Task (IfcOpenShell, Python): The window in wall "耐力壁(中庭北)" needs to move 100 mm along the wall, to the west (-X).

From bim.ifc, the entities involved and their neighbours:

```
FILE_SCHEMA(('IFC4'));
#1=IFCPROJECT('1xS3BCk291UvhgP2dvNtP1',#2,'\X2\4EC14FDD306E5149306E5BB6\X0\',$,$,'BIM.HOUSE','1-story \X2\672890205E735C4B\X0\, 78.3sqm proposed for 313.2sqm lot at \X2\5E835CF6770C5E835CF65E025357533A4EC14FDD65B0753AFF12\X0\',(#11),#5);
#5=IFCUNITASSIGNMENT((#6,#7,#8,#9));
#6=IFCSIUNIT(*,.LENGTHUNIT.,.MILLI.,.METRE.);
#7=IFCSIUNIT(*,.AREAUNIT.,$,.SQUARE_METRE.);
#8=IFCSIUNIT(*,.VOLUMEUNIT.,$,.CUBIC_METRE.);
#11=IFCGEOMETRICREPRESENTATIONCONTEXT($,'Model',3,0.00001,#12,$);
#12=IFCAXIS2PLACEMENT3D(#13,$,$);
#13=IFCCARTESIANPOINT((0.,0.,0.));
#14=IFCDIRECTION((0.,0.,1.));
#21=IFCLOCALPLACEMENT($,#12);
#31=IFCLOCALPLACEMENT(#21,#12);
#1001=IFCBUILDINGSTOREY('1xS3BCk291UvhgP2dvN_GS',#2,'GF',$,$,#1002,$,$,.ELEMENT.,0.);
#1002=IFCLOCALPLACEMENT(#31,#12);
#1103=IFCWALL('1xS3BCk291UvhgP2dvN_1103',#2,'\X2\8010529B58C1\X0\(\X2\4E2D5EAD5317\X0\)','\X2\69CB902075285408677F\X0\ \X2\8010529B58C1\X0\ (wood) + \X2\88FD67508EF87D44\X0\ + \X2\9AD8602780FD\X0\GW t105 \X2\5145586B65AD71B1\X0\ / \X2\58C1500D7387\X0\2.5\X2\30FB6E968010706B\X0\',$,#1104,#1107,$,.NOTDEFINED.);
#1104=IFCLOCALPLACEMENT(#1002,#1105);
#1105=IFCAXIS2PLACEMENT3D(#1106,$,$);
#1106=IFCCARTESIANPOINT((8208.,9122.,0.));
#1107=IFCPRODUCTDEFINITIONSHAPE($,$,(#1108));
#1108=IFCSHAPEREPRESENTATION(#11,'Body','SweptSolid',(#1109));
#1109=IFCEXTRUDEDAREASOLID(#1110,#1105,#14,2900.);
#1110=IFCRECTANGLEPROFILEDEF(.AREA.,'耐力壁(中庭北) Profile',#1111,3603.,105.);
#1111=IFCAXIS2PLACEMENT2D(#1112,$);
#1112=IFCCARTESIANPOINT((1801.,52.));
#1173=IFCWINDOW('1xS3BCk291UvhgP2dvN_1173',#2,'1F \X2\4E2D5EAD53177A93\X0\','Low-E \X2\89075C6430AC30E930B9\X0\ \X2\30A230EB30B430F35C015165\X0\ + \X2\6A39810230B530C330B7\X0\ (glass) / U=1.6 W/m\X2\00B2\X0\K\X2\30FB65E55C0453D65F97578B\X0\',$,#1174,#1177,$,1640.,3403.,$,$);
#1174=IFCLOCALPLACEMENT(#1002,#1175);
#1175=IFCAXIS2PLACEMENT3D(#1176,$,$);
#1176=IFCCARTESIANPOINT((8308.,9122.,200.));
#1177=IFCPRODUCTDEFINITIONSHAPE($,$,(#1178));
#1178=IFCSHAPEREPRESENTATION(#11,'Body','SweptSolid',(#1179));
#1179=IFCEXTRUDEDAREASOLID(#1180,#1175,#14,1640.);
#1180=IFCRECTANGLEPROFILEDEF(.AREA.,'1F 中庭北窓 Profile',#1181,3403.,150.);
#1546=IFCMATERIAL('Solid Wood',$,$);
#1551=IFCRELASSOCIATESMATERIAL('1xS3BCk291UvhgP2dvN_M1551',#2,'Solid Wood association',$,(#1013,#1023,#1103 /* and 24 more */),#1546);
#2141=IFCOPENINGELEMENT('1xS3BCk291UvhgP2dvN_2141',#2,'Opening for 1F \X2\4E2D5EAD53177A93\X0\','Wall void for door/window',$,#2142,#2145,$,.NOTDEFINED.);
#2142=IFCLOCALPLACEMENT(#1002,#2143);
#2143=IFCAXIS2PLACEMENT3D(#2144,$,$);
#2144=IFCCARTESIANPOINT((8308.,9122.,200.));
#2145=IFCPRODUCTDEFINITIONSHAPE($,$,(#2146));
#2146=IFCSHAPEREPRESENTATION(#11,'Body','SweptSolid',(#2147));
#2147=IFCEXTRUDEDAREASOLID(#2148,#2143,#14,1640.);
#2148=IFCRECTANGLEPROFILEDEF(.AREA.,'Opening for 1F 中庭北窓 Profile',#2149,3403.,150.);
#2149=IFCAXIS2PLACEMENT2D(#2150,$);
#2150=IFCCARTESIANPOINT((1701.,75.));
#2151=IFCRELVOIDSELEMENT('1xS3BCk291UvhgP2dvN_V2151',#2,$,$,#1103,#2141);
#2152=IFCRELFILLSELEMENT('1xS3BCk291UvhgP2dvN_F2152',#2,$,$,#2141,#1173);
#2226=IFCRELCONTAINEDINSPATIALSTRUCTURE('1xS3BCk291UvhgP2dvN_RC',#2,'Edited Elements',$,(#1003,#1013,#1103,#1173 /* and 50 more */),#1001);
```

```python
import ifcopenshell
import ifcopenshell.api.geometry
import ifcopenshell.util.placement

model = ifcopenshell.open("bim.ifc")

window = model.by_guid("1xS3BCk291UvhgP2dvN_1173")
opening = window.FillsVoids[0].RelatingOpeningElement
wall = opening.VoidsElements[0].RelatingBuildingElement

wall_matrix = ifcopenshell.util.placement.get_local_placement(wall.ObjectPlacement)
shift = wall_matrix[:3, 0] * -100.0
before = ifcopenshell.util.placement.get_local_placement(window.ObjectPlacement)[:3, 3].copy()

# The window is not placed relative to its opening, so move both.
for product in (opening, window):
    matrix = ifcopenshell.util.placement.get_local_placement(product.ObjectPlacement)
    matrix[:3, 3] += shift
    ifcopenshell.api.geometry.edit_object_placement(model, product=product, matrix=matrix, is_si=False)

after = ifcopenshell.util.placement.get_local_placement(window.ObjectPlacement)[:3, 3]
print("window moved by", (after - before).round(3) + 0.0)

model.write("bim_rev.ifc")
```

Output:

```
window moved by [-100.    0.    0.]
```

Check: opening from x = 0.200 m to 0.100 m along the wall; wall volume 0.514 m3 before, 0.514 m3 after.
